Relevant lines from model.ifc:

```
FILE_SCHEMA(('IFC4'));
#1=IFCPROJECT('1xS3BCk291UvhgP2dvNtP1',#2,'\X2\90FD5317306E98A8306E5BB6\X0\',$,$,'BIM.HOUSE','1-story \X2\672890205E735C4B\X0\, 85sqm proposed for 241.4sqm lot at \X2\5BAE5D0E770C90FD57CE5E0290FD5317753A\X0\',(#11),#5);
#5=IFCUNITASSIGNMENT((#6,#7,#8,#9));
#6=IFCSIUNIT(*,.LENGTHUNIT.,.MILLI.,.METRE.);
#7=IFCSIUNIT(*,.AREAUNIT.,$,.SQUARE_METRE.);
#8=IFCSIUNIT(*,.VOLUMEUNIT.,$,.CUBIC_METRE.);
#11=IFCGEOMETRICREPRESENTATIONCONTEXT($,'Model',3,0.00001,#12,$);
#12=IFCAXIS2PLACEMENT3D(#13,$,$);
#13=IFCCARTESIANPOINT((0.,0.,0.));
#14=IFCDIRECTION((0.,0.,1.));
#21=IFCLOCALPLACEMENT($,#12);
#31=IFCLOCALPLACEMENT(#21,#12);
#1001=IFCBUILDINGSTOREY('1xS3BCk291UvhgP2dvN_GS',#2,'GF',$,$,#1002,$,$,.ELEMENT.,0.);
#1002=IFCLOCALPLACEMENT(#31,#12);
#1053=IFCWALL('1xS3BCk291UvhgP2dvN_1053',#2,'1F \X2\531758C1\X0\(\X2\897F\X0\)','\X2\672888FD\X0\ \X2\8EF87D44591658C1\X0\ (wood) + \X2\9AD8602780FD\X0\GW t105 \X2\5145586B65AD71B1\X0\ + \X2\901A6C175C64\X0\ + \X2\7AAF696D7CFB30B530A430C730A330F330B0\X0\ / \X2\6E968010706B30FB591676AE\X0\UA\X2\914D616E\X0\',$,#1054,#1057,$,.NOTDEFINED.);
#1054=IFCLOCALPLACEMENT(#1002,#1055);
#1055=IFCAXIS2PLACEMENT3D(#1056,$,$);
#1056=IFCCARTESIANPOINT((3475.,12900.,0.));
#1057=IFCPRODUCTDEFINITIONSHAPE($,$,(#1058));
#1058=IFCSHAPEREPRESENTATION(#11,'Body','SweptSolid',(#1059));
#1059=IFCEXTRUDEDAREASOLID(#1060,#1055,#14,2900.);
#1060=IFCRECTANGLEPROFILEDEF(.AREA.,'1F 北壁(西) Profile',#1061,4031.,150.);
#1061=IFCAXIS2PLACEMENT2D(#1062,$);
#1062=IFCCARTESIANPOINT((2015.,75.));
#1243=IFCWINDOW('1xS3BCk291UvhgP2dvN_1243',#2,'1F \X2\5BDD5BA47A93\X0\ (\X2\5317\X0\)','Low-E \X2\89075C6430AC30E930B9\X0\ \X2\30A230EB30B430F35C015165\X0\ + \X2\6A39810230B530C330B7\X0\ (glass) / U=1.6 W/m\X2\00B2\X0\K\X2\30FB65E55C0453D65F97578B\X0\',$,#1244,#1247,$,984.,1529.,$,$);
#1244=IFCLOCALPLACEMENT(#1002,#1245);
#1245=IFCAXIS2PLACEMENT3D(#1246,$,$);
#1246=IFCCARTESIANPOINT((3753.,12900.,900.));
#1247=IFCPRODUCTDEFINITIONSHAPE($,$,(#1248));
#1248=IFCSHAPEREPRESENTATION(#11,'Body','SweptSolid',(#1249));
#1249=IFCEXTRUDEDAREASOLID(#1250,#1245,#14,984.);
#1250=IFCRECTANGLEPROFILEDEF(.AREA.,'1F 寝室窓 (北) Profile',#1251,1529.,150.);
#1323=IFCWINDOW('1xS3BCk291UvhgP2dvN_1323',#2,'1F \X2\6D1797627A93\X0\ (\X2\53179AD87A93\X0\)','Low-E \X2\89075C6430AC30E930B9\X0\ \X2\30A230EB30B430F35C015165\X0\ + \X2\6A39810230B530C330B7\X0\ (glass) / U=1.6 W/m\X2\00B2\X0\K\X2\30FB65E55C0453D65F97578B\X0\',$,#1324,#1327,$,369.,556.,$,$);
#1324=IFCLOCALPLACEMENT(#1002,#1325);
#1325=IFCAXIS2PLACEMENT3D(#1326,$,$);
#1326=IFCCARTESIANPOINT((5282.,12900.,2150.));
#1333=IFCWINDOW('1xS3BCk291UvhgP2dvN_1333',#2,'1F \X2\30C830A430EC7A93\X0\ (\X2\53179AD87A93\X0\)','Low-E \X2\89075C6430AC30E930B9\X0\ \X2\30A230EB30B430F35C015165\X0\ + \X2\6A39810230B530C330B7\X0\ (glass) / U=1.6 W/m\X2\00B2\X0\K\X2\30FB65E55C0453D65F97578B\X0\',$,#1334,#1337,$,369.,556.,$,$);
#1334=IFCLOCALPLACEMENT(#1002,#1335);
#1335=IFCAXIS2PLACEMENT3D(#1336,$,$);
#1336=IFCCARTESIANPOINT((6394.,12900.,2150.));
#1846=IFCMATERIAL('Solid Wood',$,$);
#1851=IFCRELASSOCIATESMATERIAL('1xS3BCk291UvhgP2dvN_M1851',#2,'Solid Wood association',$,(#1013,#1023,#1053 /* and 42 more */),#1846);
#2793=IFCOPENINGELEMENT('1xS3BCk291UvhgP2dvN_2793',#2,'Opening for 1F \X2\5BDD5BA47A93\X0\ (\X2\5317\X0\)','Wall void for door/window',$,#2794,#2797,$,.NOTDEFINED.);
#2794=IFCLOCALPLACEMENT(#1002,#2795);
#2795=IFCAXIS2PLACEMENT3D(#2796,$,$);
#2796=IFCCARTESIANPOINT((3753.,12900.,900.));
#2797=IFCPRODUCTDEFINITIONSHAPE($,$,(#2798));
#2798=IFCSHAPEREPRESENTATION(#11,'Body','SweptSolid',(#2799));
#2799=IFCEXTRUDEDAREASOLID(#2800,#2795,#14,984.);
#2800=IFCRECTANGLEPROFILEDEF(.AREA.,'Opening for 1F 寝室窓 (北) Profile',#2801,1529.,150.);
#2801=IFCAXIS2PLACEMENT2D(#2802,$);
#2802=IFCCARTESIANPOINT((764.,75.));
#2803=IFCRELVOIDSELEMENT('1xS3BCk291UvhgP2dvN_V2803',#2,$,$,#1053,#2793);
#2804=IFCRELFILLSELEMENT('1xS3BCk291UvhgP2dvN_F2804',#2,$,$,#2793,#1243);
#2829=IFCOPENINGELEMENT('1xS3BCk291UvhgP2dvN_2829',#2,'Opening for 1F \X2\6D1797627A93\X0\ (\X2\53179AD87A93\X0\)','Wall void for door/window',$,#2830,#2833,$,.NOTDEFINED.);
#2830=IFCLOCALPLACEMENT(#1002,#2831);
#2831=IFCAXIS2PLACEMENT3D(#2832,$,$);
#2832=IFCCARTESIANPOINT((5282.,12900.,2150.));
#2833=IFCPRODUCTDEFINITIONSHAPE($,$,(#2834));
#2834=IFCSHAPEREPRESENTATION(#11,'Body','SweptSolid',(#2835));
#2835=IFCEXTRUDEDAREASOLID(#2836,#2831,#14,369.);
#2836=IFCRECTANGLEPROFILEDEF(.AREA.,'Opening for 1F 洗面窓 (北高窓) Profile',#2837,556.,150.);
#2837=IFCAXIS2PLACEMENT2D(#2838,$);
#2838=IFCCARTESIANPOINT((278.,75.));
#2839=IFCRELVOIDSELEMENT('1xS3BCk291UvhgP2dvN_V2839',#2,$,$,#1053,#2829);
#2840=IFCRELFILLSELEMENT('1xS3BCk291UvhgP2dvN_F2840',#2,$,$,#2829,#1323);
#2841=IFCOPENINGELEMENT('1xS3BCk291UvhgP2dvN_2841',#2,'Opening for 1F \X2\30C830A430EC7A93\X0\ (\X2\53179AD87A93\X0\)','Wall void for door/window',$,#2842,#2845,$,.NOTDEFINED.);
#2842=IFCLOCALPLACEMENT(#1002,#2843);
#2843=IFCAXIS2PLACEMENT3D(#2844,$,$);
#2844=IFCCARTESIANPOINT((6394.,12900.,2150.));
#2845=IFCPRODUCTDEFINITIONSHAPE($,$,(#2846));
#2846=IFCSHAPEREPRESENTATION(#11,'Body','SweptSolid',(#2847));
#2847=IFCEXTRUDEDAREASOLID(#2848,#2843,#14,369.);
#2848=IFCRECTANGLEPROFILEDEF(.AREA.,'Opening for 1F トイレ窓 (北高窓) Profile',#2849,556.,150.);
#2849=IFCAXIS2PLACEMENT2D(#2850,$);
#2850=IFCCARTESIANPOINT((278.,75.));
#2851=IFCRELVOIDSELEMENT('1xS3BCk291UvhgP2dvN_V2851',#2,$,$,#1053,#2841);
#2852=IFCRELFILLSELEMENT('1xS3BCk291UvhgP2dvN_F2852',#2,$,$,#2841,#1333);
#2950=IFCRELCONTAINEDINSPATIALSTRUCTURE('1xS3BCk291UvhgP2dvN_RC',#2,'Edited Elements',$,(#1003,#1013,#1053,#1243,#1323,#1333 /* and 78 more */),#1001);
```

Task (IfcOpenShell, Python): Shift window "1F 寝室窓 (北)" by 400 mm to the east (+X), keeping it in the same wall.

```python
import ifcopenshell
import ifcopenshell.api.geometry
import ifcopenshell.util.placement
import ifcopenshell.util.unit

model = ifcopenshell.open("model.ifc")
unit_scale = ifcopenshell.util.unit.calculate_unit_scale(model)

window = model.by_guid("1xS3BCk291UvhgP2dvN_1243")
opening = window.FillsVoids[0].RelatingOpeningElement
wall = opening.VoidsElements[0].RelatingBuildingElement

wall_matrix = ifcopenshell.util.placement.get_local_placement(wall.ObjectPlacement)
shift = wall_matrix[:3, 0] * 0.4 / unit_scale
before = ifcopenshell.util.placement.get_local_placement(window.ObjectPlacement)[:3, 3].copy()

# The window is not placed relative to its opening, so move both.
for product in (opening, window):
    matrix = ifcopenshell.util.placement.get_local_placement(product.ObjectPlacement)
    matrix[:3, 3] += shift
    ifcopenshell.api.geometry.edit_object_placement(model, product=product, matrix=matrix, is_si=False)

after = ifcopenshell.util.placement.get_local_placement(window.ObjectPlacement)[:3, 3]
print("window moved by", (after - before).round(3) + 0.0)

model.write("model-out.ifc")
```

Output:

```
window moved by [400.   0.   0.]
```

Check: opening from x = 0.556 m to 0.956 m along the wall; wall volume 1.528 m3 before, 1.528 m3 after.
